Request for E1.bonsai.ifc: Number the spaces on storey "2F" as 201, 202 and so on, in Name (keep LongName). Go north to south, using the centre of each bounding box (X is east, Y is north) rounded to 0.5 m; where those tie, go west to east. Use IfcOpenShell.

First a look at what the model holds.

```python
import ifcopenshell
import ifcopenshell.util.element
import ifcopenshell.util.placement

model = ifcopenshell.open("E1.bonsai.ifc")
print(model.schema)
storey = next(s for s in model.by_type("IfcBuildingStorey") if s.Name == "2F")
spaces = [e for e in ifcopenshell.util.element.get_decomposition(storey) if e.is_a("IfcSpace")]
for e in sorted(spaces, key=lambda e: e.id()):
    origin = ifcopenshell.util.placement.get_local_placement(e.ObjectPlacement)[:3, 3]
    print(e.id(), e.Name, e.LongName, origin.round(2) + 0.0, sep=" | ")
```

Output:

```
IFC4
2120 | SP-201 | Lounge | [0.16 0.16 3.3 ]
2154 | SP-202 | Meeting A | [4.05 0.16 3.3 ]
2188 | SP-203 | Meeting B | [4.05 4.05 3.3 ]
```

```python
import ifcopenshell
import ifcopenshell.geom
import ifcopenshell.util.element
import ifcopenshell.util.shape

model = ifcopenshell.open("E1.bonsai.ifc")
settings = ifcopenshell.geom.settings()
settings.set("use-world-coords", True)


def centre(element):
    shape = ifcopenshell.geom.create_shape(settings, element)
    return ifcopenshell.util.shape.get_bbox_centroid(shape.geometry)


storey = next(s for s in model.by_type("IfcBuildingStorey") if s.Name == "2F")
spaces = [e for e in ifcopenshell.util.element.get_decomposition(storey) if e.is_a("IfcSpace")]

# Insertion points can sit at a corner or the storey origin, so sort by the geometry (in metres).
centres = {e: centre(e) for e in spaces}
spaces.sort(key=lambda e: (-round(centres[e][1] / 0.5), centres[e][0]))

for i, e in enumerate(spaces, start=1):
    number = f"2{i:02d}"
    e.Name = number
    print(e.id(), number)

model.write("E1.bonsai-out.ifc")
```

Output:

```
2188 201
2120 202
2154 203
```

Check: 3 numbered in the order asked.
